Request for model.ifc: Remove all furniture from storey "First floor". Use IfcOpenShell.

First a look at what the model holds.

```python
import ifcopenshell
import ifcopenshell.util.element

model = ifcopenshell.open("model.ifc")
print(model.schema)
storey = next(s for s in model.by_type("IfcBuildingStorey") if s.Name == "First floor")
furniture = [e for e in ifcopenshell.util.element.get_decomposition(storey) if e.is_a("IfcFurnishingElement")]
seen = {}
for e in furniture:
    element_type = ifcopenshell.util.element.get_type(e)
    name = element_type.Name if element_type not in (None, e) else None
    seen[name] = seen.get(name, 0) + 1
for name, count in sorted(seen.items(), key=str):
    print(count, "x", name)
```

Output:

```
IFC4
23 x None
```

```python
import ifcopenshell
import ifcopenshell.api.root
import ifcopenshell.util.element

model = ifcopenshell.open("model.ifc")

storey = next(s for s in model.by_type("IfcBuildingStorey") if s.Name == "First floor")
furniture = [e for e in ifcopenshell.util.element.get_decomposition(storey) if e.is_a("IfcFurnishingElement")]

for e in furniture:
    ifcopenshell.api.root.remove_product(model, product=e)
print(len(furniture), "removed")

model.write("model-out.ifc")
```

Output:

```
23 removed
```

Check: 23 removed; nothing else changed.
